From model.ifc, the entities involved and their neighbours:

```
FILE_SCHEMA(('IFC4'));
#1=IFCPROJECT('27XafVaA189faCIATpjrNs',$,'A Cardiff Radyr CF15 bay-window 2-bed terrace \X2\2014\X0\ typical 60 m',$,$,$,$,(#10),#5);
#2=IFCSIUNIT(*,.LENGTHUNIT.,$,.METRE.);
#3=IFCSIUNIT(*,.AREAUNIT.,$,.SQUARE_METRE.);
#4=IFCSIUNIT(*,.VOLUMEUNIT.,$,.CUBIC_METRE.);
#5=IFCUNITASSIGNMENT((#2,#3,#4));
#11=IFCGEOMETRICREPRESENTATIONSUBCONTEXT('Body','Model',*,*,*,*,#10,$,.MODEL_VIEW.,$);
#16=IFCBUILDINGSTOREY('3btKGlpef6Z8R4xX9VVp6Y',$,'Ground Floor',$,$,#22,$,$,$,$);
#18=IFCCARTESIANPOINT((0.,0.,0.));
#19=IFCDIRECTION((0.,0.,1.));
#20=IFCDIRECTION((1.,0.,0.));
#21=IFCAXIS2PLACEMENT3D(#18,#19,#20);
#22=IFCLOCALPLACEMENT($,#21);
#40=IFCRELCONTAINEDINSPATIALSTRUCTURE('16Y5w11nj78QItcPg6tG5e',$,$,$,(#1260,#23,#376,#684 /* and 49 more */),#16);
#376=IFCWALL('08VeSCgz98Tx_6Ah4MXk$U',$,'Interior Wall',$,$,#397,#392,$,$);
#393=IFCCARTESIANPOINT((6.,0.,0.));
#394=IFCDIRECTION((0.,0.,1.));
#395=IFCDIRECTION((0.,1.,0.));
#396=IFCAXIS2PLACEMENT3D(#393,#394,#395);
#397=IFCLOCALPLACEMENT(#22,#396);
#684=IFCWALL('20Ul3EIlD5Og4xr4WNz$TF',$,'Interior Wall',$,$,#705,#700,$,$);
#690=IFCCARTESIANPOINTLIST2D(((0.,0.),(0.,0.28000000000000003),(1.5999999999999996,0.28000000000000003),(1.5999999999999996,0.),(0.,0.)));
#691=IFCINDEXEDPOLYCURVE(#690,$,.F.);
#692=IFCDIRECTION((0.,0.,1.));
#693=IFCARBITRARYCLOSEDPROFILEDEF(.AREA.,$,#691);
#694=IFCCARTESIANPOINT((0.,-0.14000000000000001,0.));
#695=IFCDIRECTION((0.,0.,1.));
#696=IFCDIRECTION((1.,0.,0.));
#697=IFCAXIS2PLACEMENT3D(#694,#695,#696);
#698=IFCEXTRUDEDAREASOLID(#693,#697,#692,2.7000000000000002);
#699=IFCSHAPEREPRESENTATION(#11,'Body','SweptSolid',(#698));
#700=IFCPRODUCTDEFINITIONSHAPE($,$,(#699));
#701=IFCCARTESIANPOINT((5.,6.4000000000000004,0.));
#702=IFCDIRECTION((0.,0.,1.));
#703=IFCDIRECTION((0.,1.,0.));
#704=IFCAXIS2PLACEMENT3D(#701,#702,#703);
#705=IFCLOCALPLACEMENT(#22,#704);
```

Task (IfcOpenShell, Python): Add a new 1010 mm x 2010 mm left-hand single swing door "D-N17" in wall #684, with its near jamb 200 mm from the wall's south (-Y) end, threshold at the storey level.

```python
import numpy as np
import ifcopenshell
import ifcopenshell.api.feature
import ifcopenshell.api.geometry
import ifcopenshell.api.root
import ifcopenshell.api.spatial
import ifcopenshell.geom
import ifcopenshell.util.element
import ifcopenshell.util.placement
import ifcopenshell.util.representation
import ifcopenshell.util.shape
import ifcopenshell.util.unit

model = ifcopenshell.open("model.ifc")
unit_scale = ifcopenshell.util.unit.calculate_unit_scale(model)
settings = ifcopenshell.geom.settings()


def volume(element):
    """Net volume in cubic metres, openings subtracted."""
    shape = ifcopenshell.geom.create_shape(settings, element)
    return ifcopenshell.util.shape.get_volume(shape.geometry)


wall = model.by_id(684)
storey = ifcopenshell.util.element.get_container(wall, ifc_class="IfcBuildingStorey")
context = ifcopenshell.util.representation.get_context(model, "Model", "Body", "MODEL_VIEW")
before = volume(wall)

width, height, from_end, sill = 1.01, 2.01, 0.2, 0.0  # metres

# The wall runs along its own X axis, and the end named is its -X end.
wall_shape = ifcopenshell.geom.create_shape(settings, wall)
x, y, z = ifcopenshell.util.shape.get_vertices(wall_shape.geometry).T
start = x.min() + from_end
face, thickness = float(y.min()), float(y.max() - y.min())
wall_matrix = ifcopenshell.util.placement.get_local_placement(wall.ObjectPlacement)
level = ifcopenshell.util.placement.get_local_placement(storey.ObjectPlacement)[2, 3]


def in_wall(x, y):
    """Placement at x, y metres in the wall's axes, at sill height."""
    matrix = wall_matrix.copy()
    matrix[:, 3] = wall_matrix @ np.array([x / unit_scale, y / unit_scale, 0.0, 1.0])
    matrix[2, 3] = level + sill / unit_scale
    return matrix


# Opening: a box that overshoots both wall faces by 50 mm.
opening = ifcopenshell.api.root.create_entity(model, ifc_class="IfcOpeningElement", predefined_type="OPENING")
box = ifcopenshell.api.geometry.add_wall_representation(
    model, context=context, length=width, height=height, thickness=thickness + 0.1
)
ifcopenshell.api.geometry.assign_representation(model, product=opening, representation=box)
ifcopenshell.api.geometry.edit_object_placement(model, product=opening, matrix=in_wall(start, face - 0.05), is_si=False)
ifcopenshell.api.feature.add_feature(model, feature=opening, element=wall)

door = ifcopenshell.api.root.create_entity(model, ifc_class="IfcDoor", name="D-N17", predefined_type="DOOR")
door.OverallWidth, door.OverallHeight = width / unit_scale, height / unit_scale
door.OperationType = "SINGLE_SWING_LEFT"
body = ifcopenshell.api.geometry.add_door_representation(
    model,
    context=context,
    overall_width=door.OverallWidth,
    overall_height=door.OverallHeight,
    operation_type="SINGLE_SWING_LEFT",
    lining_properties={"LiningDepth": thickness / unit_scale, "ThresholdDepth": thickness / unit_scale},
)
ifcopenshell.api.geometry.assign_representation(model, product=door, representation=body)
ifcopenshell.api.spatial.assign_container(model, products=[door], relating_structure=storey)
ifcopenshell.api.feature.add_filling(model, opening=opening, element=door)

# The lining spans the wall, so the door starts at the wall face.
ifcopenshell.api.geometry.edit_object_placement(model, product=door, matrix=in_wall(start, face), is_si=False)

after = volume(wall)

print(f"wall volume {before:.3f} -> {after:.3f} m3")

model.write("model_edited.ifc")
```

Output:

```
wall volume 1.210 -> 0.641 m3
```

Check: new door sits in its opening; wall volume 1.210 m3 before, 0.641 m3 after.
